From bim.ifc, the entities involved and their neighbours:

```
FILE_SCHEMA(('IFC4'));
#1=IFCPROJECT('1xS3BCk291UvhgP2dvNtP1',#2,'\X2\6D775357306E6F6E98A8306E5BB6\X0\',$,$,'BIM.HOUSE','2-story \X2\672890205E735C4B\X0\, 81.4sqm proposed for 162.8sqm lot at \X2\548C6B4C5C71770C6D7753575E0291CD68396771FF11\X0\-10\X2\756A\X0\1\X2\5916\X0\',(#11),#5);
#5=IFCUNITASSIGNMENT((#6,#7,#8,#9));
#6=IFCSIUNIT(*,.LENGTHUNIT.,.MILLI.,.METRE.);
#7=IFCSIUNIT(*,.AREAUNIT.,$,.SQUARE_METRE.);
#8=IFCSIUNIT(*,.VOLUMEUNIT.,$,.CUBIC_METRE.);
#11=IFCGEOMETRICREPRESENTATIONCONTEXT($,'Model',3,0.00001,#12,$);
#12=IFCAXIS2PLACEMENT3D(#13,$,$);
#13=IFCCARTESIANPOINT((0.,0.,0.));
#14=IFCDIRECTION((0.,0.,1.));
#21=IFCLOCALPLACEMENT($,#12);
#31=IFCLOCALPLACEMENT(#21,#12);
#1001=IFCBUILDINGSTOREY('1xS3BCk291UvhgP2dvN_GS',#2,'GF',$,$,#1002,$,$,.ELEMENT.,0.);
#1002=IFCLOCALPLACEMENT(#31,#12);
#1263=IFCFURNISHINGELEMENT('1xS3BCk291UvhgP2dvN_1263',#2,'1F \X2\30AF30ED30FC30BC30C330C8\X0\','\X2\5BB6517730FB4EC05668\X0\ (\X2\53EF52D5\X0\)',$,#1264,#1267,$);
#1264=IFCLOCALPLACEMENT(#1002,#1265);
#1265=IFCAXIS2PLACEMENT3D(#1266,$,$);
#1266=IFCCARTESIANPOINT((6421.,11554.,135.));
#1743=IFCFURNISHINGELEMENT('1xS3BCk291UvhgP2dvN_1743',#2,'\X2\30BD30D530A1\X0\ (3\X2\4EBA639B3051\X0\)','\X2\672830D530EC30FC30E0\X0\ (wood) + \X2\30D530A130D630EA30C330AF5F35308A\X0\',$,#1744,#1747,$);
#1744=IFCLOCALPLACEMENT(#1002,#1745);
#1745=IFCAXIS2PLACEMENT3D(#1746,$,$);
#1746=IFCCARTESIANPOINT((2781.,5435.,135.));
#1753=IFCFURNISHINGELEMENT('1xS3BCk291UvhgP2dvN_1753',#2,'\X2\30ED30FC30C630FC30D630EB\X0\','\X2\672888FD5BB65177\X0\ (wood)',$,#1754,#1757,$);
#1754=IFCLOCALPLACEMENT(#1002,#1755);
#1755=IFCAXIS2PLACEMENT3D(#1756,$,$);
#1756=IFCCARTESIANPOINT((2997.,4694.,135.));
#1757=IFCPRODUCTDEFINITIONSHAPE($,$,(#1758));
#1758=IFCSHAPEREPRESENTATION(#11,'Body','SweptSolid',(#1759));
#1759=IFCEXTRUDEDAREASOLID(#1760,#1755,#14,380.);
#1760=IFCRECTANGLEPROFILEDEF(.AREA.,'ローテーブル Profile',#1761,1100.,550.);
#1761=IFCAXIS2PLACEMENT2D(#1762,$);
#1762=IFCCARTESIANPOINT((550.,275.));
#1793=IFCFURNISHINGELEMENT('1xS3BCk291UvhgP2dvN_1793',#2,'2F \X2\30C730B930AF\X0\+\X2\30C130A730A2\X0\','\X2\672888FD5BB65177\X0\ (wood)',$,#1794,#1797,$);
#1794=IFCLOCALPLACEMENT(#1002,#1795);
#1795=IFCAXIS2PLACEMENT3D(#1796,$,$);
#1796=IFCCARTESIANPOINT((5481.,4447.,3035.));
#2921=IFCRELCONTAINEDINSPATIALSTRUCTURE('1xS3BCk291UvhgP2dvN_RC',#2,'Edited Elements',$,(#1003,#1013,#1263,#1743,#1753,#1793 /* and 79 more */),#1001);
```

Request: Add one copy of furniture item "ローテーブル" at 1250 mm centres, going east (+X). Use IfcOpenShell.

```python
import numpy as np
import ifcopenshell
import ifcopenshell.api.geometry
import ifcopenshell.api.root
import ifcopenshell.util.element
import ifcopenshell.util.placement

model = ifcopenshell.open("bim.ifc")


def reuse_history(source, copy):
    """copy_class also copies each property set's owner history, people and application; keep the originals."""
    for rel in copy.IsDefinedBy:
        if rel.is_a("IfcRelDefinesByProperties") and (history := rel.RelatingPropertyDefinition.OwnerHistory):
            rel.RelatingPropertyDefinition.OwnerHistory = source.OwnerHistory
            ifcopenshell.util.element.remove_deep2(model, history)


source = model.by_guid("1xS3BCk291UvhgP2dvN_1753")
base = ifcopenshell.util.placement.get_local_placement(source.ObjectPlacement)
step = np.array([1.0, 0.0, 0.0]) * 1250.0

for i in range(1, 2):
    copy = ifcopenshell.api.root.copy_class(model, product=source)
    copy.Representation = ifcopenshell.util.element.copy_deep(
        model, source.Representation, exclude=["IfcGeometricRepresentationContext", "IfcRepresentationMap"]
    )
    reuse_history(source, copy)
    matrix = base.copy()
    matrix[:3, 3] += i * step
    print("added at", matrix[:3, 3].round(3) + 0.0)
    ifcopenshell.api.geometry.edit_object_placement(model, product=copy, matrix=matrix, is_si=False)

model.write("bim-out.ifc")
```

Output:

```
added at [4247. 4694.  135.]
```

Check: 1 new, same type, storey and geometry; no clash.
